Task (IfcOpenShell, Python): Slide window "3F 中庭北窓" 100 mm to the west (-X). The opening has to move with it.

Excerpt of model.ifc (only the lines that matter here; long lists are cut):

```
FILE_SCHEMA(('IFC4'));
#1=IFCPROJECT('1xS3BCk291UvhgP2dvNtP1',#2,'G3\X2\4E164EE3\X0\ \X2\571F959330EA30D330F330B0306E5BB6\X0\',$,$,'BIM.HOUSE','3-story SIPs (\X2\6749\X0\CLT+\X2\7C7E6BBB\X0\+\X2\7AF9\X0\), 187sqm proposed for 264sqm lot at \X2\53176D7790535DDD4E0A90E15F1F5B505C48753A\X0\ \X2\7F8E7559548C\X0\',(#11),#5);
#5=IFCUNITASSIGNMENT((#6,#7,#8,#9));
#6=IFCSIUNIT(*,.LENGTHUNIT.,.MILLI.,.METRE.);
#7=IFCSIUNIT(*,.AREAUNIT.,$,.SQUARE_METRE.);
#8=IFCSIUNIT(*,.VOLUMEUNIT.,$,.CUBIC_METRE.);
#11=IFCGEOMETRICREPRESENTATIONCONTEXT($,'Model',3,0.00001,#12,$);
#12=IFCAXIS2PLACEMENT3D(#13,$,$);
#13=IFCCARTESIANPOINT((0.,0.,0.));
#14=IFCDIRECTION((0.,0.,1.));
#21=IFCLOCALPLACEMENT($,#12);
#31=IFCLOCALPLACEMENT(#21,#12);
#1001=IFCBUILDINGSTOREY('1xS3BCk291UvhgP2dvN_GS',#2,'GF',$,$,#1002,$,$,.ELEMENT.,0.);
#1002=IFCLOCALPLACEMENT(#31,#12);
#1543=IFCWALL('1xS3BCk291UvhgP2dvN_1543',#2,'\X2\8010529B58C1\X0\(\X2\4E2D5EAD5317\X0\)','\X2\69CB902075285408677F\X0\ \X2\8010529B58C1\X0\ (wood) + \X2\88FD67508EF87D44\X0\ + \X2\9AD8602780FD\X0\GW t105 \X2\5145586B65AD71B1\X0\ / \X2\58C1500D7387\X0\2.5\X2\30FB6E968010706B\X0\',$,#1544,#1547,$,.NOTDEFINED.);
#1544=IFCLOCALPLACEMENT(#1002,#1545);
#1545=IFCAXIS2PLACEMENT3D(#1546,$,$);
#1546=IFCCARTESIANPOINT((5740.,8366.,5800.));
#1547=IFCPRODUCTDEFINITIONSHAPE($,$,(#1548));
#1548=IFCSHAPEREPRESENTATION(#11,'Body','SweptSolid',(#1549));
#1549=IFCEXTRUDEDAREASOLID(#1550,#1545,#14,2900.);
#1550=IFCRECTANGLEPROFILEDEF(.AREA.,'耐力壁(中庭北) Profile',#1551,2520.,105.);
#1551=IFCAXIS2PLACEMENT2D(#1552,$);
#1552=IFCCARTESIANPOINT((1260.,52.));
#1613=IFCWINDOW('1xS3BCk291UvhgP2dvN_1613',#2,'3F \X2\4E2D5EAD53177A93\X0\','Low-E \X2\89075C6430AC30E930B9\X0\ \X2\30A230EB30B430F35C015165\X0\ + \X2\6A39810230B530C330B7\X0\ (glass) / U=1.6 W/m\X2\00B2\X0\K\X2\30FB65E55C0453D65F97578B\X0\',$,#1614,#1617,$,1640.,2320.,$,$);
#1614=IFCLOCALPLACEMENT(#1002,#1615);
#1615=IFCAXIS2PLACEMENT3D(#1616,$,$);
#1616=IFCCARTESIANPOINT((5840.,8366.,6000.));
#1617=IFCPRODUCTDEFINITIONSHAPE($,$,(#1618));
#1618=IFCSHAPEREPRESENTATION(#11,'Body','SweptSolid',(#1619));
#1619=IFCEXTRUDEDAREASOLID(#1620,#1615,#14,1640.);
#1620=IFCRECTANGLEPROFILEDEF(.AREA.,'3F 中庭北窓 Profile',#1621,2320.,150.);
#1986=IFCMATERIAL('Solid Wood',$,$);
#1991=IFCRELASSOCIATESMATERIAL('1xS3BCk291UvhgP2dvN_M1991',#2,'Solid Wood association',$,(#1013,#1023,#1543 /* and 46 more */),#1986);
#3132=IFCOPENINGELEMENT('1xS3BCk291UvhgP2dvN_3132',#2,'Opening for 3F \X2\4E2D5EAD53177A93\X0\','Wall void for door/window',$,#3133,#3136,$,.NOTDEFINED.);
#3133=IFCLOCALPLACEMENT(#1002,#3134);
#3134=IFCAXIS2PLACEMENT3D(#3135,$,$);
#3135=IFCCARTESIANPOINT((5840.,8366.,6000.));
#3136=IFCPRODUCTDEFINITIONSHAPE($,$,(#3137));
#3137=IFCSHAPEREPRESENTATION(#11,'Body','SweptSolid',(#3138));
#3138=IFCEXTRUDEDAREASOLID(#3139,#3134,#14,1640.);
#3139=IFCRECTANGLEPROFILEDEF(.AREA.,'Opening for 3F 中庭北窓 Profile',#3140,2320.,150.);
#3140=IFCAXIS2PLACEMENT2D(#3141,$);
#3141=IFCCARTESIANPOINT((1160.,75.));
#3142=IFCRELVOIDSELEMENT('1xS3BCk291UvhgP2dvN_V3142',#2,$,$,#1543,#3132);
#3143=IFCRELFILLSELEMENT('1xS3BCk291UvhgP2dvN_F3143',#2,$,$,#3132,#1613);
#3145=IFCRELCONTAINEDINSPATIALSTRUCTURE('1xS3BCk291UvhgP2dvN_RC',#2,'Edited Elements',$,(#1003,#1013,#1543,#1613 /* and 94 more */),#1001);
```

```python
import ifcopenshell
import ifcopenshell.api.geometry
import ifcopenshell.util.placement

model = ifcopenshell.open("model.ifc")

window = model.by_guid("1xS3BCk291UvhgP2dvN_1613")
opening = window.FillsVoids[0].RelatingOpeningElement
wall = opening.VoidsElements[0].RelatingBuildingElement

wall_matrix = ifcopenshell.util.placement.get_local_placement(wall.ObjectPlacement)
shift = wall_matrix[:3, 0] * -100.0
before = ifcopenshell.util.placement.get_local_placement(window.ObjectPlacement)[:3, 3].copy()

# The window is not placed relative to its opening, so move both.
for product in (opening, window):
    matrix = ifcopenshell.util.placement.get_local_placement(product.ObjectPlacement)
    matrix[:3, 3] += shift
    ifcopenshell.api.geometry.edit_object_placement(model, product=product, matrix=matrix, is_si=False)

after = ifcopenshell.util.placement.get_local_placement(window.ObjectPlacement)[:3, 3]
print("window moved by", (after - before).round(3) + 0.0)

model.write("model_v2.ifc")
```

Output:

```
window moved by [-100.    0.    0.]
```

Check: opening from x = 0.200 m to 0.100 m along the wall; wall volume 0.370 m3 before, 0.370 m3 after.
